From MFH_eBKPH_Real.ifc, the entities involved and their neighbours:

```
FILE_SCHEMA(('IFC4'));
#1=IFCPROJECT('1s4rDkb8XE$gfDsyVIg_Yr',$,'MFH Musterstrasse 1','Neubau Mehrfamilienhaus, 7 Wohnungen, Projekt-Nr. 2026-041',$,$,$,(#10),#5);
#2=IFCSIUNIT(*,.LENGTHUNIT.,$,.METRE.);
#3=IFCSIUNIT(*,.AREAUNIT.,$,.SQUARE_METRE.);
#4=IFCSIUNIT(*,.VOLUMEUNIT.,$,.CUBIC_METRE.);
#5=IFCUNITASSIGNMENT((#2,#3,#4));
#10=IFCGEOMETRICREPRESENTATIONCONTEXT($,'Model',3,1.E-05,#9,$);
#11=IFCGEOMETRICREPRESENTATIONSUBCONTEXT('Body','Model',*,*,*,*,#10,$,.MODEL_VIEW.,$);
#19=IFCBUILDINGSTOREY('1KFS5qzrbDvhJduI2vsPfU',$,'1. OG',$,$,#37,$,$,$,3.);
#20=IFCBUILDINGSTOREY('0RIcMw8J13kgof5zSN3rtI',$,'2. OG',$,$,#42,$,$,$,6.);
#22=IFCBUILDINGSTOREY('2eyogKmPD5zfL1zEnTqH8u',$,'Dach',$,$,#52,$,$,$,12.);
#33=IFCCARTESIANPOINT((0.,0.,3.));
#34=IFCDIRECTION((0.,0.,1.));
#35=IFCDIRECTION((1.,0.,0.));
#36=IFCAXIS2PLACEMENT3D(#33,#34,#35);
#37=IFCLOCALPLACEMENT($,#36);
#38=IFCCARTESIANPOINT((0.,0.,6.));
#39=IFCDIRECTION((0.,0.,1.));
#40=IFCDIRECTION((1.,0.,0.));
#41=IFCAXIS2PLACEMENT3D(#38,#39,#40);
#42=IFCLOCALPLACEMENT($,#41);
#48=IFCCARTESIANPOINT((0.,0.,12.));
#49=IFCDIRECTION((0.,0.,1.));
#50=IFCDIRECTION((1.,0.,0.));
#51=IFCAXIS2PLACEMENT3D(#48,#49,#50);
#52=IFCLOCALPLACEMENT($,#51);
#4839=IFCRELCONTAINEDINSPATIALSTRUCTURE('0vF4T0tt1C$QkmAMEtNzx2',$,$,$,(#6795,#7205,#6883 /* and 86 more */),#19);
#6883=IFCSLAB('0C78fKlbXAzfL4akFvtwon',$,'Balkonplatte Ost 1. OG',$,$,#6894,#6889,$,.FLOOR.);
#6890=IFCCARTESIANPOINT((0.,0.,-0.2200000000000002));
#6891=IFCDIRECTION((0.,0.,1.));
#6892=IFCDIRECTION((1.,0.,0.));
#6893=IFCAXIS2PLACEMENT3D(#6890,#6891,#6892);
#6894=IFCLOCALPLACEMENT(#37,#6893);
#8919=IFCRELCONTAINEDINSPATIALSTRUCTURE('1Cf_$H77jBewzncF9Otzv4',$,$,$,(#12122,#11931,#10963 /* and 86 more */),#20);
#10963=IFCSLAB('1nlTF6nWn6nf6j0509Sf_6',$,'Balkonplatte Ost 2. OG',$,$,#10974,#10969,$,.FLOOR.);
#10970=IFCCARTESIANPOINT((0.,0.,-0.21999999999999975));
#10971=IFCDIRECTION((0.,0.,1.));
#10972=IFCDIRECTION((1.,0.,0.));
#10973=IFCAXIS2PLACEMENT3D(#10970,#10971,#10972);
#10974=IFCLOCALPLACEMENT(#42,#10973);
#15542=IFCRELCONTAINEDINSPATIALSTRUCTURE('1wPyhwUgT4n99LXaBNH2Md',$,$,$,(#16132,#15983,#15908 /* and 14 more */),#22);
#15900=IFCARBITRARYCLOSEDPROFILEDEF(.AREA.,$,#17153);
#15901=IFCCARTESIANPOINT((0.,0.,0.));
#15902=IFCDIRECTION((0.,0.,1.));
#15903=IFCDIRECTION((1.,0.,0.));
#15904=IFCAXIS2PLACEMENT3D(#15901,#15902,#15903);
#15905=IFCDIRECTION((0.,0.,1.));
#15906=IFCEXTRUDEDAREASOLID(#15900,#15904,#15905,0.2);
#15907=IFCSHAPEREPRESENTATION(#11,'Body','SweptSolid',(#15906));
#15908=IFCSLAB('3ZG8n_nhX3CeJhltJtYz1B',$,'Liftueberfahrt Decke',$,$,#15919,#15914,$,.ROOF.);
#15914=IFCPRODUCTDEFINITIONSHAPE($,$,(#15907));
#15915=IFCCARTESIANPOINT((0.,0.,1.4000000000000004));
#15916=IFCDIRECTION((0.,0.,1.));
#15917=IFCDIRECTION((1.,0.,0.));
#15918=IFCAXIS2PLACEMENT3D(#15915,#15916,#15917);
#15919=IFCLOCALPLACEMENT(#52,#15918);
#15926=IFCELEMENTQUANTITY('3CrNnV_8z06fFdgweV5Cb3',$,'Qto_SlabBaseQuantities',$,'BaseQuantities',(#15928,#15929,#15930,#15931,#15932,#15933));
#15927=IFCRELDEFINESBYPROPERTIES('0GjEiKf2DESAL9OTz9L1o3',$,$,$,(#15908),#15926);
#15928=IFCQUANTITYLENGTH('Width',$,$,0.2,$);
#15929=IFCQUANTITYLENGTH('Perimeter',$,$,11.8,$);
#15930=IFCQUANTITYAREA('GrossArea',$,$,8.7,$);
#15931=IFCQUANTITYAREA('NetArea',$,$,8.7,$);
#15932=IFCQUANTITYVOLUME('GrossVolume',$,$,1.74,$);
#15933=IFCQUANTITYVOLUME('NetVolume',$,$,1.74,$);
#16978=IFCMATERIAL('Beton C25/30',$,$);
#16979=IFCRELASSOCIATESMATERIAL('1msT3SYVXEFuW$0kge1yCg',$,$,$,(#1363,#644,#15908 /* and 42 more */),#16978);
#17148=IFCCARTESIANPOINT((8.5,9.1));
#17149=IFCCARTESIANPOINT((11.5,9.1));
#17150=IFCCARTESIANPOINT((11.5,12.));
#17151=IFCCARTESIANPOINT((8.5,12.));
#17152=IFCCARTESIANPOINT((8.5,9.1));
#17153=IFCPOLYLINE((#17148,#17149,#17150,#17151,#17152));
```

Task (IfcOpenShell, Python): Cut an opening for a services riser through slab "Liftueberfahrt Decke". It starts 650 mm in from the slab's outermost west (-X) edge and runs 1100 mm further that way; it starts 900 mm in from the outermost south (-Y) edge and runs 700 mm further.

```python
import numpy as np
import ifcopenshell
import ifcopenshell.api.feature
import ifcopenshell.api.geometry
import ifcopenshell.api.pset
import ifcopenshell.api.root
import ifcopenshell.geom
import ifcopenshell.util.element
import ifcopenshell.util.placement
import ifcopenshell.util.representation
import ifcopenshell.util.shape
import ifcopenshell.util.unit

model = ifcopenshell.open("MFH_eBKPH_Real.ifc")
unit_scale = ifcopenshell.util.unit.calculate_unit_scale(model)
area_scale = ifcopenshell.util.unit.calculate_unit_scale(model, "AREAUNIT")
volume_scale = ifcopenshell.util.unit.calculate_unit_scale(model, "VOLUMEUNIT")
settings = ifcopenshell.geom.settings()


def volume(element):
    """Net volume in cubic metres, openings subtracted."""
    shape = ifcopenshell.geom.create_shape(settings, element)
    return ifcopenshell.util.shape.get_volume(shape.geometry)


slab = model.by_guid("3ZG8n_nhX3CeJhltJtYz1B")
before = volume(slab)

# Extent in the slab's own axes, in metres. The edges named are its -X and -Y sides.
slab_shape = ifcopenshell.geom.create_shape(settings, slab)
vertices = ifcopenshell.util.shape.get_vertices(slab_shape.geometry)
x_min, y_min, bottom = vertices.min(axis=0)
top = vertices[:, 2].max()

opening = ifcopenshell.api.root.create_entity(model, ifc_class="IfcOpeningElement", name="Services riser opening", predefined_type="OPENING")
context = ifcopenshell.util.representation.get_context(model, "Model", "Body", "MODEL_VIEW")
width, depth = 1.1, 0.7
outline = [(0.0, 0.0), (width, 0.0), (width, depth), (0.0, depth), (0.0, 0.0)]
# Overshoot both faces by 50 mm so the cut is clean.
shape = ifcopenshell.api.geometry.add_slab_representation(
    model, context=context, depth=top - bottom + 0.1, polyline=outline
)
ifcopenshell.api.geometry.assign_representation(model, product=opening, representation=shape)

matrix = ifcopenshell.util.placement.get_local_placement(slab.ObjectPlacement)
matrix[:, 3] = matrix @ np.append(np.array([x_min + 0.65, y_min + 0.9, bottom - 0.05]) / unit_scale, 1.0)
ifcopenshell.api.geometry.edit_object_placement(model, product=opening, matrix=matrix, is_si=False)
ifcopenshell.api.feature.add_feature(model, feature=opening, element=slab)

after = volume(slab)

# Update the slab's stored quantities.
qto = model.by_id(ifcopenshell.util.element.get_pset(slab, "Qto_SlabBaseQuantities", should_inherit=False)["id"])
ifcopenshell.api.pset.edit_qto(model, qto=qto, properties={
    "NetArea": after / (top - bottom) / area_scale,
    "NetVolume": after / volume_scale,
})

print(f"slab volume {before:.3f} -> {after:.3f} m3")

model.write("MFH_eBKPH_Real_v2.ifc")
```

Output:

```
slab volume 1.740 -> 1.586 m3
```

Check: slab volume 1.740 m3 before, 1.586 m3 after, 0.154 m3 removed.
